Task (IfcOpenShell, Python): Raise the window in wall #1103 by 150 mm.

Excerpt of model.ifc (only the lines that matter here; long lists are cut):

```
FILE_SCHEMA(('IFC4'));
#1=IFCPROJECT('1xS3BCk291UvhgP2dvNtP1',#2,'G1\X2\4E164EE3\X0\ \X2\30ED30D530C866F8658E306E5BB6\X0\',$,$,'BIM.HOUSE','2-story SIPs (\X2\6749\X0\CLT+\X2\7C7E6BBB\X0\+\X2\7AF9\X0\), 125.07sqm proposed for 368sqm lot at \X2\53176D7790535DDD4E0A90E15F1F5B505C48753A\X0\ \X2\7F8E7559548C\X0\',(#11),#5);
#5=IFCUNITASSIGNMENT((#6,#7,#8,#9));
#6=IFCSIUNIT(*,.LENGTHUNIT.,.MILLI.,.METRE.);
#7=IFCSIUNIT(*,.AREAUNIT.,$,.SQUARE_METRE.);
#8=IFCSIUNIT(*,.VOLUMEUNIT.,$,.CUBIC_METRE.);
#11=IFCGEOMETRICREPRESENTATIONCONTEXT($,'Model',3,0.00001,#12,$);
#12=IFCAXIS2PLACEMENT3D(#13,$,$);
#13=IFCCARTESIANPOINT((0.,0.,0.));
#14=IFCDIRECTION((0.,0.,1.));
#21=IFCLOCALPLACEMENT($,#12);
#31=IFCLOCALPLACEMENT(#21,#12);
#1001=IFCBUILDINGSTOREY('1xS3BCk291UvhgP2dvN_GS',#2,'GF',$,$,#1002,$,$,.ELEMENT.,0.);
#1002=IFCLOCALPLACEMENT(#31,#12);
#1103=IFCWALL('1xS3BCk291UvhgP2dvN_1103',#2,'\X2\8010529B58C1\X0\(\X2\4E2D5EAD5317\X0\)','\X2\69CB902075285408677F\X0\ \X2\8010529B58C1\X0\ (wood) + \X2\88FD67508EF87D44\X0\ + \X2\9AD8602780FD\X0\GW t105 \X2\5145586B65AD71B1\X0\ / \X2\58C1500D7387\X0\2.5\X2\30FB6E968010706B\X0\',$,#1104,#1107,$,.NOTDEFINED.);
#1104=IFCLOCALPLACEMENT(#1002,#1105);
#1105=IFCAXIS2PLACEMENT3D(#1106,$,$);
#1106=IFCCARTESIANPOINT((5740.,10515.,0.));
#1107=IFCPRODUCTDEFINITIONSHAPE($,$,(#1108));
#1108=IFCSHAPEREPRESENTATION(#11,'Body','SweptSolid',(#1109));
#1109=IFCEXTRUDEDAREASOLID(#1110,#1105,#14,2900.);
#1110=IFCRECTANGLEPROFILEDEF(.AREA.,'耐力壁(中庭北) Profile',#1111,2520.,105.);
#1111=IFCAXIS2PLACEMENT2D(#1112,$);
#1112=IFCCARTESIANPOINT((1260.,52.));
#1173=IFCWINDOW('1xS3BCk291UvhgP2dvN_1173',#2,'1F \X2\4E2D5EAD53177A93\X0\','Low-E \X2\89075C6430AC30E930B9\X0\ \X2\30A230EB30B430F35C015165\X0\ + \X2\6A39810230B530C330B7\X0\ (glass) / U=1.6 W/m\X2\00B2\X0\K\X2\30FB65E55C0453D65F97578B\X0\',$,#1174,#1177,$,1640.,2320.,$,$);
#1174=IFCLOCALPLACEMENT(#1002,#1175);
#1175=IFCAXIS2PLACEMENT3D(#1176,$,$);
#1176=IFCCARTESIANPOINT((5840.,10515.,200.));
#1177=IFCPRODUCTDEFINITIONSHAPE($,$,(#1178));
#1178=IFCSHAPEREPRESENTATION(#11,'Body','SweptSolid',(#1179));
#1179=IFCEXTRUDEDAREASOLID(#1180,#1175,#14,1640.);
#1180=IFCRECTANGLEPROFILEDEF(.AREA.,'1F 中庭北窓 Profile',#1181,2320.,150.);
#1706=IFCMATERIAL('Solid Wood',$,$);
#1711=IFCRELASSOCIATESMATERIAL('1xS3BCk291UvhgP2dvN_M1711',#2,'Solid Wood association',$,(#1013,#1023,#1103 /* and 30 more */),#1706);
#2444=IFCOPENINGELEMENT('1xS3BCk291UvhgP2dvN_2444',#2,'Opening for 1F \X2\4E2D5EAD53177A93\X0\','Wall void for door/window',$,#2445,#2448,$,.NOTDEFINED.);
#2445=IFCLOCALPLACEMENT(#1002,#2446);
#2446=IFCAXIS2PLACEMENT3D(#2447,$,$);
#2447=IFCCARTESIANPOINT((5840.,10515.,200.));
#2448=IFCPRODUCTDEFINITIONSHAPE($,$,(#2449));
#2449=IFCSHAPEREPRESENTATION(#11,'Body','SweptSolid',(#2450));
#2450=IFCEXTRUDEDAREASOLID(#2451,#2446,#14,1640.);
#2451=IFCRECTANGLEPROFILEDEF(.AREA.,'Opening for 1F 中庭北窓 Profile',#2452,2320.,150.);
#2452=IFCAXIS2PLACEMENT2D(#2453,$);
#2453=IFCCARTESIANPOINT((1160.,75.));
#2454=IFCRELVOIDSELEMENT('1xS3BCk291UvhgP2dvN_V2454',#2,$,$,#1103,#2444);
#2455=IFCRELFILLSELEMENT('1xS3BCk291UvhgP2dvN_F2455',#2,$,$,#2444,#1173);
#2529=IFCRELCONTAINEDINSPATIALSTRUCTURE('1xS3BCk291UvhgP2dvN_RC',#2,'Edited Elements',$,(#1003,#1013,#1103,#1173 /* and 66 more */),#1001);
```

```python
import numpy as np
import ifcopenshell
import ifcopenshell.api.geometry
import ifcopenshell.util.placement
import ifcopenshell.util.unit

model = ifcopenshell.open("model.ifc")
unit_scale = ifcopenshell.util.unit.calculate_unit_scale(model)

window = model.by_guid("1xS3BCk291UvhgP2dvN_1173")
opening = window.FillsVoids[0].RelatingOpeningElement
dz = 150.0

shift = np.array([0.0, 0.0, dz])
# The window is not placed relative to its opening, so move both.
for product in (opening, window):
    matrix = ifcopenshell.util.placement.get_local_placement(product.ObjectPlacement)
    matrix[:3, 3] += shift
    ifcopenshell.api.geometry.edit_object_placement(model, product=product, matrix=matrix, is_si=False)

print(f"moved by {dz * unit_scale:+.3f} m")

model.write("model-out.ifc")
```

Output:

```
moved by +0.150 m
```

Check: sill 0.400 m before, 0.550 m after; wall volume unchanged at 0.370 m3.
